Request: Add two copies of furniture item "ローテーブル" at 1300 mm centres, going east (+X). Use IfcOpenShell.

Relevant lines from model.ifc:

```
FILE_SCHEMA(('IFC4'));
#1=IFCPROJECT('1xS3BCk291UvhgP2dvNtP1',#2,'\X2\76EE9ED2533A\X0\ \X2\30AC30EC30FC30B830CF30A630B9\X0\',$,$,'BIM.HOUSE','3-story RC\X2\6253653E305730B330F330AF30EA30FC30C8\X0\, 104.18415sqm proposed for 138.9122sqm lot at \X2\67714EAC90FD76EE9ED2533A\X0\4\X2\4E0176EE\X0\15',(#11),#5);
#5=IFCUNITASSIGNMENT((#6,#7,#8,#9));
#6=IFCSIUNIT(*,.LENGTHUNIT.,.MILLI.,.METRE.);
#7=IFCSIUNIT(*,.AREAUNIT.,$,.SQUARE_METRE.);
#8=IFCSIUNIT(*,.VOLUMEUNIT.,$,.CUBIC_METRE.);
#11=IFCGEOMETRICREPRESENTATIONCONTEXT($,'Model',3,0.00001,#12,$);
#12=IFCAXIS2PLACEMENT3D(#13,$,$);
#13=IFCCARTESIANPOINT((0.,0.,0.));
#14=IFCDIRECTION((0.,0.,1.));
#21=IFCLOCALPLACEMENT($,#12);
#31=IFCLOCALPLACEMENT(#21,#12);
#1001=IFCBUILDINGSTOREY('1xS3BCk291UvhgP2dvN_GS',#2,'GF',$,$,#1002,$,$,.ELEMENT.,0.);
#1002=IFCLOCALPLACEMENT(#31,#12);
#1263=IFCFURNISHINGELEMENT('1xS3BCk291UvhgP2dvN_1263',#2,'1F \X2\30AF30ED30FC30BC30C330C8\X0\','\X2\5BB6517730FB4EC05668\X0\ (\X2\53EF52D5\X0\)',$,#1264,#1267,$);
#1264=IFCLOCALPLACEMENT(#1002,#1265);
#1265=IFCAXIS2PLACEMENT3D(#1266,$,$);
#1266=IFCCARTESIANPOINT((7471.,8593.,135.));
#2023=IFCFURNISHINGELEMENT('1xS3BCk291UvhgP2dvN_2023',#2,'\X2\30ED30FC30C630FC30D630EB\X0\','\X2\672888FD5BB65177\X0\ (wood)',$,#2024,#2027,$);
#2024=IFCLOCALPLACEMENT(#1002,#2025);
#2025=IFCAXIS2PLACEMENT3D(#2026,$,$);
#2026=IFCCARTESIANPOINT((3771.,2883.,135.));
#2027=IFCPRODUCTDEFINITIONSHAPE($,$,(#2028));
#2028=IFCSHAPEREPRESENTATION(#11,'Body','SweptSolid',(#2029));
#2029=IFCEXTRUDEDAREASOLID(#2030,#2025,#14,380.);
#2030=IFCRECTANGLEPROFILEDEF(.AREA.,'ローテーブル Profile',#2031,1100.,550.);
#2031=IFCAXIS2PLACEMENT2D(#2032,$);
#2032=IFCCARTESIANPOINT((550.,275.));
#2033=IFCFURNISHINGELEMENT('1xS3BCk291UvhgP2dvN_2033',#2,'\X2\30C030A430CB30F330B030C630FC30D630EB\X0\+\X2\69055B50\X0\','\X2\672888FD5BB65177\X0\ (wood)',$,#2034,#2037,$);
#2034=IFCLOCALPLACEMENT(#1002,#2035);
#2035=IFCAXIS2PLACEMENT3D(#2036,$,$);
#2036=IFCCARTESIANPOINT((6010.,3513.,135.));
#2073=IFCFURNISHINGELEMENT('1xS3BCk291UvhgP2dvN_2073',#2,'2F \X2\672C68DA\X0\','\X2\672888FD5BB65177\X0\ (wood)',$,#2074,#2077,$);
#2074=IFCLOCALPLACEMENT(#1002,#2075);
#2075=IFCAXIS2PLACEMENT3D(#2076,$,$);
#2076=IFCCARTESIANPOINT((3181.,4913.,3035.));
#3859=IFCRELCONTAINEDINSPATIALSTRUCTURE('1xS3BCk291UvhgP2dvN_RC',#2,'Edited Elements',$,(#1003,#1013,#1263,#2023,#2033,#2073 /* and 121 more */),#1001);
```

```python
import numpy as np
import ifcopenshell
import ifcopenshell.api.geometry
import ifcopenshell.api.root
import ifcopenshell.util.element
import ifcopenshell.util.placement
import ifcopenshell.util.unit

model = ifcopenshell.open("model.ifc")
unit_scale = ifcopenshell.util.unit.calculate_unit_scale(model)


def reuse_history(source, copy):
    """copy_class also copies each property set's owner history, people and application; keep the originals."""
    for rel in copy.IsDefinedBy:
        if rel.is_a("IfcRelDefinesByProperties") and (history := rel.RelatingPropertyDefinition.OwnerHistory):
            rel.RelatingPropertyDefinition.OwnerHistory = source.OwnerHistory
            ifcopenshell.util.element.remove_deep2(model, history)


source = model.by_guid("1xS3BCk291UvhgP2dvN_2023")
base = ifcopenshell.util.placement.get_local_placement(source.ObjectPlacement)
step = np.array([1.0, 0.0, 0.0]) * 1.3 / unit_scale

for i in range(1, 3):
    copy = ifcopenshell.api.root.copy_class(model, product=source)
    copy.Representation = ifcopenshell.util.element.copy_deep(
        model, source.Representation, exclude=["IfcGeometricRepresentationContext", "IfcRepresentationMap"]
    )
    reuse_history(source, copy)
    matrix = base.copy()
    matrix[:3, 3] += i * step
    print("added at", matrix[:3, 3].round(3) + 0.0)
    ifcopenshell.api.geometry.edit_object_placement(model, product=copy, matrix=matrix, is_si=False)

model.write("model_v2.ifc")
```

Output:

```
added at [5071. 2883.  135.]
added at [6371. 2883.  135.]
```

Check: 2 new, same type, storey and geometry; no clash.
